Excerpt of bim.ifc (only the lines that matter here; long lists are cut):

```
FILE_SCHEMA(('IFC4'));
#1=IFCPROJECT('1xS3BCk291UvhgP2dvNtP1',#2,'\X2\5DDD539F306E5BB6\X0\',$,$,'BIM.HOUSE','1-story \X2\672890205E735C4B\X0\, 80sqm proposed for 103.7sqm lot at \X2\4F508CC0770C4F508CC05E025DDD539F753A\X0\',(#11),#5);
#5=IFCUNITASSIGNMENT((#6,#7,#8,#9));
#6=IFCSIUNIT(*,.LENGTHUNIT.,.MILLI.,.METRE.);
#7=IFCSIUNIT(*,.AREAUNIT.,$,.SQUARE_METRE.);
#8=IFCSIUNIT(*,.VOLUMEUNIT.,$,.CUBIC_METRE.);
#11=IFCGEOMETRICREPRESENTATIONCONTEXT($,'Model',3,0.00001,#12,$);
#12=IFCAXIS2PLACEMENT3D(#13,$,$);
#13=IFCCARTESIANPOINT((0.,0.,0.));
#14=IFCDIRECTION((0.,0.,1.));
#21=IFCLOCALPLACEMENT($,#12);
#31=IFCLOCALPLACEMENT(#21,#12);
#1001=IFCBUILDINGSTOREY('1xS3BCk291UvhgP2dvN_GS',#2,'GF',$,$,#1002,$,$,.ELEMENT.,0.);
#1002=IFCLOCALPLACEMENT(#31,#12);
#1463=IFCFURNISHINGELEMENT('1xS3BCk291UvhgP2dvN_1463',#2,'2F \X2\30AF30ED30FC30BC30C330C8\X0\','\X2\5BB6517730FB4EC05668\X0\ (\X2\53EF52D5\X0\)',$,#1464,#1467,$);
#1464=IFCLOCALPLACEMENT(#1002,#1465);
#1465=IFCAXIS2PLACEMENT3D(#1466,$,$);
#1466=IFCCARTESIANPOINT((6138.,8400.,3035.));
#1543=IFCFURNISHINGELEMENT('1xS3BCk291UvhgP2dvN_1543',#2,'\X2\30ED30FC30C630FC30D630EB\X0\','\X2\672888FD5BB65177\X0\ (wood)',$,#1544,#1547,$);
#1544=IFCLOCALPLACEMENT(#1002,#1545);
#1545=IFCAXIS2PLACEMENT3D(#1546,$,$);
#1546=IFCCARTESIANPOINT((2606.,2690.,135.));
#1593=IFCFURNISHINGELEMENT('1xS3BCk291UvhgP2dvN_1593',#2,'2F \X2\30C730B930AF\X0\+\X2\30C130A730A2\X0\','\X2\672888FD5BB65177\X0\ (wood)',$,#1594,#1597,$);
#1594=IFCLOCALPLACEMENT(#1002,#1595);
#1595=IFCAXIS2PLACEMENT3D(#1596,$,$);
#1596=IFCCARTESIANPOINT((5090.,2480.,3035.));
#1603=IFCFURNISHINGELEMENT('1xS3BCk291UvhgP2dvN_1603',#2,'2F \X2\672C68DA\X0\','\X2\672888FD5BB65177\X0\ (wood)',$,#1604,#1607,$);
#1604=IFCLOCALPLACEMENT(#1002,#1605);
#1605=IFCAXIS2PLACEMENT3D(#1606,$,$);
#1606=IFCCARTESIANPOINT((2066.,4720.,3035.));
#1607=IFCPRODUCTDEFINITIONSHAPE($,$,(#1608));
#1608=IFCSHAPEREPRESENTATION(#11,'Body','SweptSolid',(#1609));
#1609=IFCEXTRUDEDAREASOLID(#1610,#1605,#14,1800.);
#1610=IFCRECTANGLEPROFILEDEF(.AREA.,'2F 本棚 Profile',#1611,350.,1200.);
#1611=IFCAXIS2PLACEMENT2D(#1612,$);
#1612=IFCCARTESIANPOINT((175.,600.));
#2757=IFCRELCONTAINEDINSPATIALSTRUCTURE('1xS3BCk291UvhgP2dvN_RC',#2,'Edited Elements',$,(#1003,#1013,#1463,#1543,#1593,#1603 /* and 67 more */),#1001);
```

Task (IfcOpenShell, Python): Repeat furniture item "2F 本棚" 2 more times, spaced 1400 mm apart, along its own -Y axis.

```python
import ifcopenshell
import ifcopenshell.api.geometry
import ifcopenshell.api.root
import ifcopenshell.util.element
import ifcopenshell.util.placement

model = ifcopenshell.open("bim.ifc")


def reuse_history(source, copy):
    """copy_class also copies each property set's owner history, people and application; keep the originals."""
    for rel in copy.IsDefinedBy:
        if rel.is_a("IfcRelDefinesByProperties") and (history := rel.RelatingPropertyDefinition.OwnerHistory):
            rel.RelatingPropertyDefinition.OwnerHistory = source.OwnerHistory
            ifcopenshell.util.element.remove_deep2(model, history)


source = model.by_id(1603)
base = ifcopenshell.util.placement.get_local_placement(source.ObjectPlacement)
step = -base[:3, 1] * 1400.0

for i in range(1, 3):
    copy = ifcopenshell.api.root.copy_class(model, product=source)
    copy.Representation = ifcopenshell.util.element.copy_deep(
        model, source.Representation, exclude=["IfcGeometricRepresentationContext", "IfcRepresentationMap"]
    )
    reuse_history(source, copy)
    matrix = base.copy()
    matrix[:3, 3] += i * step
    print("added at", matrix[:3, 3].round(3) + 0.0)
    ifcopenshell.api.geometry.edit_object_placement(model, product=copy, matrix=matrix, is_si=False)

model.write("bim_v2.ifc")
```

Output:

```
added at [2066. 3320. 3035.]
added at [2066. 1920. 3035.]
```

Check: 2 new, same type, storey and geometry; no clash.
